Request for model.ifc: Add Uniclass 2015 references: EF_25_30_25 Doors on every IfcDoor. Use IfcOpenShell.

First a look at what the model holds.

```python
import ifcopenshell

model = ifcopenshell.open("model.ifc")
print(model.schema)
print("classifications:", [c.Name for c in model.by_type("IfcClassification")])
for ifc_class in ("IfcDoor", "IfcRoof", "IfcStair", "IfcWall", "IfcWindow"):
    print(ifc_class, len(model.by_type(ifc_class)))
```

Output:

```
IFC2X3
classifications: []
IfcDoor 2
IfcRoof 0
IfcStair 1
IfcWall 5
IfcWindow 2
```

```python
import ifcopenshell
import ifcopenshell.api.classification

model = ifcopenshell.open("model.ifc")

# IFC2X3 requires Source and Edition and has no link from the project to the system.
system = model.create_entity("IfcClassification", Source="NBS", Edition="2015", Name="Uniclass 2015")

codes = {
    "IfcDoor": ("EF_25_30_25", "Doors"),
}
for ifc_class, (code, name) in codes.items():
    products = model.by_type(ifc_class)
    ifcopenshell.api.classification.add_reference(
        model, products=products, classification=system, identification=code, name=name
    )
    print(code, len(products))

model.write("model_updated.ifc")
```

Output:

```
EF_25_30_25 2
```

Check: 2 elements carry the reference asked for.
